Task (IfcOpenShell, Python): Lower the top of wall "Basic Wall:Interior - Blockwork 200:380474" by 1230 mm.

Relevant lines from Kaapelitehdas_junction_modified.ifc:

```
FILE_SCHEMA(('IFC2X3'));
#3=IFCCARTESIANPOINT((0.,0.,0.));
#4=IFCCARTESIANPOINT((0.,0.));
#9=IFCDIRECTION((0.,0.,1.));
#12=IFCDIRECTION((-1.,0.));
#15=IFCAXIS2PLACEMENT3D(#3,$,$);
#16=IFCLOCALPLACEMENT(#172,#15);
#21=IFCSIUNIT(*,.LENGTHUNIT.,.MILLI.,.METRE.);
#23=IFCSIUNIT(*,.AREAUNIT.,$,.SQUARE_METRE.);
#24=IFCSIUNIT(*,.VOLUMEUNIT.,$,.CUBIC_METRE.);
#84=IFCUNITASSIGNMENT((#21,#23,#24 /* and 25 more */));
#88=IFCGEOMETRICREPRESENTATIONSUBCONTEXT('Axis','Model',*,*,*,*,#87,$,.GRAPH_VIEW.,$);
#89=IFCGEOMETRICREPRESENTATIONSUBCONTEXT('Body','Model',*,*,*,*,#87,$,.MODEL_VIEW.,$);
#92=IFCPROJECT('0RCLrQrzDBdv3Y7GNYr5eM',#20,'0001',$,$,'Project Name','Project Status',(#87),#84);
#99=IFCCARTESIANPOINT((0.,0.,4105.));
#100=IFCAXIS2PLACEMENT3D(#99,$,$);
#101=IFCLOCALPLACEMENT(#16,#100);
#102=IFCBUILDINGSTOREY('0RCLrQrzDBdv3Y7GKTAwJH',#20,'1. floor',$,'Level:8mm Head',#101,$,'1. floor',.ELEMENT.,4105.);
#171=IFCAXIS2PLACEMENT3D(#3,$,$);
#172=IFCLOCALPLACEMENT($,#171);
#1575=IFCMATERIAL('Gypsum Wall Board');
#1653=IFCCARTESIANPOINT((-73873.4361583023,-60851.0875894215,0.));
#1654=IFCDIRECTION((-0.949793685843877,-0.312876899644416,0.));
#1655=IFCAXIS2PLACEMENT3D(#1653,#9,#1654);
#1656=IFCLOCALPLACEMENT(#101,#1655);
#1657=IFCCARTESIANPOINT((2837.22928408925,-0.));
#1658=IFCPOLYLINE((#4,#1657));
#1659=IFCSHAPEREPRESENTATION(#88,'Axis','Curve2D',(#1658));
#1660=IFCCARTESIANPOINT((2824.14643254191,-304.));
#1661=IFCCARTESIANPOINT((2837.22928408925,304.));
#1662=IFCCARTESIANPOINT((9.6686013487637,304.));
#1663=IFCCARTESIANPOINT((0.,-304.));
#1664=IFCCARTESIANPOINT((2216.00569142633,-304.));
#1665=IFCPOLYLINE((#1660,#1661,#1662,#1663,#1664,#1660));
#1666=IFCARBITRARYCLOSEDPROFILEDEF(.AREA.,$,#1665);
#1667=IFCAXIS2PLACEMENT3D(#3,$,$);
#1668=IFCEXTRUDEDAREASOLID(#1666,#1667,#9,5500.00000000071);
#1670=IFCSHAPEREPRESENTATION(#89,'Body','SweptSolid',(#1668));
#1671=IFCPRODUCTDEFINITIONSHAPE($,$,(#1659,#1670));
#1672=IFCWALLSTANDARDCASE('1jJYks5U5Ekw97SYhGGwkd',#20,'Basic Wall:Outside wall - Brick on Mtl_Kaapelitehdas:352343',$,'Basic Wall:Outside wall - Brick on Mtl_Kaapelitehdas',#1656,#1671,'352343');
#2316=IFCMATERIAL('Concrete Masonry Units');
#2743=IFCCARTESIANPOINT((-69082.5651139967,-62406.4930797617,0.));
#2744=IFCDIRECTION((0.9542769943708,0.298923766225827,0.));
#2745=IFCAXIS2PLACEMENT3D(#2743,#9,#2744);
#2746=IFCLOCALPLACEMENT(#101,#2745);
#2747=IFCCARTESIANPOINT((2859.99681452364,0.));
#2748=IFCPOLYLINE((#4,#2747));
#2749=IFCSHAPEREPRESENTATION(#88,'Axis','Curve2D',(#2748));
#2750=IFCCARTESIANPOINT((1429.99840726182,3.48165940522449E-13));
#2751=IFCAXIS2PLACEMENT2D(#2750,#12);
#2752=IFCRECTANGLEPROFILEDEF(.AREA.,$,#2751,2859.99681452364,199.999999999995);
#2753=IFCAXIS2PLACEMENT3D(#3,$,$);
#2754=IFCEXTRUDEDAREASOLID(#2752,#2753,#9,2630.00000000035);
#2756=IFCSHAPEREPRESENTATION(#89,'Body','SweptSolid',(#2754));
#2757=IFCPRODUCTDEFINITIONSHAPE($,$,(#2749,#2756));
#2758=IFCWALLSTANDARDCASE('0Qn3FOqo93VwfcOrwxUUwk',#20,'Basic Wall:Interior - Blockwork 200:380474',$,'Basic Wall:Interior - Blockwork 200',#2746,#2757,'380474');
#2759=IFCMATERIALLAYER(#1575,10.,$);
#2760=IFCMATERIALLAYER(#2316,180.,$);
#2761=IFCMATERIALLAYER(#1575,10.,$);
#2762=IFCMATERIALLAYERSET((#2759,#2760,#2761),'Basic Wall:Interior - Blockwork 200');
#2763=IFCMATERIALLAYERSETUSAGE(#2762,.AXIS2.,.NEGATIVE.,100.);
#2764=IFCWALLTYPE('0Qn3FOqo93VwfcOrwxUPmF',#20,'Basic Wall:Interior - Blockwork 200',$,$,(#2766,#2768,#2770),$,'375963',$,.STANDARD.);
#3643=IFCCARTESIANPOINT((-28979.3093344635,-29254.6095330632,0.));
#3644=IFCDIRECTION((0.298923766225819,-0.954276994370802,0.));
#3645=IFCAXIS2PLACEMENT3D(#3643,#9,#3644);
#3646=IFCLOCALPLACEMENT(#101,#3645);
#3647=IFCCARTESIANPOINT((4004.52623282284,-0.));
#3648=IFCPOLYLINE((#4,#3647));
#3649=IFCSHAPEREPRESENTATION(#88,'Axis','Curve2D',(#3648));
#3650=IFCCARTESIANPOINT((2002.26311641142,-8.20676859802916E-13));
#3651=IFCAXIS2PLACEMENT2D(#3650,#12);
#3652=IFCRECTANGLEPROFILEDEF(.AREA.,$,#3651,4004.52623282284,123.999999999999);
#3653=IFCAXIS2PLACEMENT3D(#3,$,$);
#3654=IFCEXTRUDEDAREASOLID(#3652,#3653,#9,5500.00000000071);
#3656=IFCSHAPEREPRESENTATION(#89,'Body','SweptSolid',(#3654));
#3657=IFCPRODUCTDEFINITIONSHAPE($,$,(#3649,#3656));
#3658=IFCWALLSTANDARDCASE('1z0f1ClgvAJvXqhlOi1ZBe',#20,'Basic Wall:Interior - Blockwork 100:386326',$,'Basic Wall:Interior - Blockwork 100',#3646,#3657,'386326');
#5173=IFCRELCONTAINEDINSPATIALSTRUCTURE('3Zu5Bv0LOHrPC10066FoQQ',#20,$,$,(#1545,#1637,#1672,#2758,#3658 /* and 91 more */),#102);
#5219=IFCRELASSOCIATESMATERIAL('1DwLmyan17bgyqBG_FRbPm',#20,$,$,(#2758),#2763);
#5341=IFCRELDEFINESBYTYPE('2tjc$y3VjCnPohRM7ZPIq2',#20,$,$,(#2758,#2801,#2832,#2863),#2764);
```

```python
import ifcopenshell
import ifcopenshell.geom
import ifcopenshell.util.representation
import ifcopenshell.util.shape
import ifcopenshell.util.unit

model = ifcopenshell.open("Kaapelitehdas_junction_modified.ifc")
unit_scale = ifcopenshell.util.unit.calculate_unit_scale(model)
settings = ifcopenshell.geom.settings()


def volume(element):
    """Net volume in cubic metres, openings subtracted."""
    shape = ifcopenshell.geom.create_shape(settings, element)
    return ifcopenshell.util.shape.get_volume(shape.geometry)


wall = model.by_guid("0Qn3FOqo93VwfcOrwxUUwk")
before = volume(wall)

body = ifcopenshell.util.representation.get_representation(wall, "Model", "Body")
solid = body.Items[0]
old_height = solid.Depth
solid.Depth -= 1.23 / unit_scale
after = volume(wall)

print(f"height {old_height:g} -> {solid.Depth:g}, volume {before:.3f} -> {after:.3f} m3")

model.write("Kaapelitehdas_junction_modified-out.ifc")
```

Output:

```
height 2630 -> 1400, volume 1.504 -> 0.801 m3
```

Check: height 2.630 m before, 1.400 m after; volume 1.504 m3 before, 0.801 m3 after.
